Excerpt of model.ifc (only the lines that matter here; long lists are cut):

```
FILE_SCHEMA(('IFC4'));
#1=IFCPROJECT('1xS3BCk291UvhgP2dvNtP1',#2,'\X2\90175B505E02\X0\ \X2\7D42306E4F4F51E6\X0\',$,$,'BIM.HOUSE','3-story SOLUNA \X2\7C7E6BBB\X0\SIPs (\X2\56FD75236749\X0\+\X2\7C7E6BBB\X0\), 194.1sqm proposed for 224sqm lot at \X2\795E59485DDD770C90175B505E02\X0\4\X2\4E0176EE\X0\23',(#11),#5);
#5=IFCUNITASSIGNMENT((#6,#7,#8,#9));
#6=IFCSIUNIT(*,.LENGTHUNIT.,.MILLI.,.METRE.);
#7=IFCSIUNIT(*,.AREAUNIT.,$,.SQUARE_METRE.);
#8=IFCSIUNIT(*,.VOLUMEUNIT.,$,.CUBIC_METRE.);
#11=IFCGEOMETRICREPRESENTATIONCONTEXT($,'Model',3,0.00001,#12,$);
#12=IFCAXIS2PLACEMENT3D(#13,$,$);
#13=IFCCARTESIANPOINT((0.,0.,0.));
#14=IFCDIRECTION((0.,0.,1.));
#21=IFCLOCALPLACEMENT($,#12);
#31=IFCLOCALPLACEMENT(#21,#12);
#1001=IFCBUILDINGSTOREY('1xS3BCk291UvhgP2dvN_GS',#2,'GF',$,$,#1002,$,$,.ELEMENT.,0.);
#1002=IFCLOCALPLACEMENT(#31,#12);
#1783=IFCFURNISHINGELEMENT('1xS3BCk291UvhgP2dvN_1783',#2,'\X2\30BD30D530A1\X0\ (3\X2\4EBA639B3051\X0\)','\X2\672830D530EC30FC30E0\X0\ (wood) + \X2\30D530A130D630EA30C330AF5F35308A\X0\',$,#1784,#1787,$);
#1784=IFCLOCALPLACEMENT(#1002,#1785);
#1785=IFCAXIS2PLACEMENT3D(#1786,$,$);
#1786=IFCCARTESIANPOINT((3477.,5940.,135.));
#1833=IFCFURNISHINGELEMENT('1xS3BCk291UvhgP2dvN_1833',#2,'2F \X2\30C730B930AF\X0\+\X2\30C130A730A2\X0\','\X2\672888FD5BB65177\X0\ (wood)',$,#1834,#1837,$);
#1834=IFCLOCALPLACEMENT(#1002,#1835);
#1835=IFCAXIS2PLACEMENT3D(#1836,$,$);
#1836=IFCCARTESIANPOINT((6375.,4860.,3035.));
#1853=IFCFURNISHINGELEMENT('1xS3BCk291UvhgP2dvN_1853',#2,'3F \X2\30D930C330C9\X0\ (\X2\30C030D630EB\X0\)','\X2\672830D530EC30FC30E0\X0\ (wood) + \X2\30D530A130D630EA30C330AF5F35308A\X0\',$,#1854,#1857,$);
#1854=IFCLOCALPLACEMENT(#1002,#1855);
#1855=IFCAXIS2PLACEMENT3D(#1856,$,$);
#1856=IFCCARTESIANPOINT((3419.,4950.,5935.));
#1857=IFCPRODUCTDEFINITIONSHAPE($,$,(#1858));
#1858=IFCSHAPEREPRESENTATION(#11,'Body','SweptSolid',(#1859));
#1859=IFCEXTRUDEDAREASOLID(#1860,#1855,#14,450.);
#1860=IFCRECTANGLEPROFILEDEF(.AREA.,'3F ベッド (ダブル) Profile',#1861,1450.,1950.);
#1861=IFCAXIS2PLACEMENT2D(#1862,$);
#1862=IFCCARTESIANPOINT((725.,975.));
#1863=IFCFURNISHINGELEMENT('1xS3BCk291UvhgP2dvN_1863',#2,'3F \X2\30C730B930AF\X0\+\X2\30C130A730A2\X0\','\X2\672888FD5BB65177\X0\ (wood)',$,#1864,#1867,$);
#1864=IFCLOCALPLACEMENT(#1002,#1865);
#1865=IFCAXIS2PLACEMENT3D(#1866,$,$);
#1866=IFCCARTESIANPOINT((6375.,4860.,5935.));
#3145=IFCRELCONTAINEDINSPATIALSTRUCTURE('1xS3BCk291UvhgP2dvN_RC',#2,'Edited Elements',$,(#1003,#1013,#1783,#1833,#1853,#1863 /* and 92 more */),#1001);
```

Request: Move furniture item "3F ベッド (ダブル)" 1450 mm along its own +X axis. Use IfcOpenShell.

```python
import ifcopenshell
import ifcopenshell.api.geometry
import ifcopenshell.util.placement
import ifcopenshell.util.unit

model = ifcopenshell.open("model.ifc")
unit_scale = ifcopenshell.util.unit.calculate_unit_scale(model)

item = model.by_guid("1xS3BCk291UvhgP2dvN_1853")
matrix = ifcopenshell.util.placement.get_local_placement(item.ObjectPlacement)
matrix[:3, 3] += matrix[:3, 0] * 1.45 / unit_scale
ifcopenshell.api.geometry.edit_object_placement(model, product=item, matrix=matrix, is_si=False)

print(ifcopenshell.util.placement.get_local_placement(item.ObjectPlacement).round(3) + 0.0)

model.write("model_v2.ifc")
```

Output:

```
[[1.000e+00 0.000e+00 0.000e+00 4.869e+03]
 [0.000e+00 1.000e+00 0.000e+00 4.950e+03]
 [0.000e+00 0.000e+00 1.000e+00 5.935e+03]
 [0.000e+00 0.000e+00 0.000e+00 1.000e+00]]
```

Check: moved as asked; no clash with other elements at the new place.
